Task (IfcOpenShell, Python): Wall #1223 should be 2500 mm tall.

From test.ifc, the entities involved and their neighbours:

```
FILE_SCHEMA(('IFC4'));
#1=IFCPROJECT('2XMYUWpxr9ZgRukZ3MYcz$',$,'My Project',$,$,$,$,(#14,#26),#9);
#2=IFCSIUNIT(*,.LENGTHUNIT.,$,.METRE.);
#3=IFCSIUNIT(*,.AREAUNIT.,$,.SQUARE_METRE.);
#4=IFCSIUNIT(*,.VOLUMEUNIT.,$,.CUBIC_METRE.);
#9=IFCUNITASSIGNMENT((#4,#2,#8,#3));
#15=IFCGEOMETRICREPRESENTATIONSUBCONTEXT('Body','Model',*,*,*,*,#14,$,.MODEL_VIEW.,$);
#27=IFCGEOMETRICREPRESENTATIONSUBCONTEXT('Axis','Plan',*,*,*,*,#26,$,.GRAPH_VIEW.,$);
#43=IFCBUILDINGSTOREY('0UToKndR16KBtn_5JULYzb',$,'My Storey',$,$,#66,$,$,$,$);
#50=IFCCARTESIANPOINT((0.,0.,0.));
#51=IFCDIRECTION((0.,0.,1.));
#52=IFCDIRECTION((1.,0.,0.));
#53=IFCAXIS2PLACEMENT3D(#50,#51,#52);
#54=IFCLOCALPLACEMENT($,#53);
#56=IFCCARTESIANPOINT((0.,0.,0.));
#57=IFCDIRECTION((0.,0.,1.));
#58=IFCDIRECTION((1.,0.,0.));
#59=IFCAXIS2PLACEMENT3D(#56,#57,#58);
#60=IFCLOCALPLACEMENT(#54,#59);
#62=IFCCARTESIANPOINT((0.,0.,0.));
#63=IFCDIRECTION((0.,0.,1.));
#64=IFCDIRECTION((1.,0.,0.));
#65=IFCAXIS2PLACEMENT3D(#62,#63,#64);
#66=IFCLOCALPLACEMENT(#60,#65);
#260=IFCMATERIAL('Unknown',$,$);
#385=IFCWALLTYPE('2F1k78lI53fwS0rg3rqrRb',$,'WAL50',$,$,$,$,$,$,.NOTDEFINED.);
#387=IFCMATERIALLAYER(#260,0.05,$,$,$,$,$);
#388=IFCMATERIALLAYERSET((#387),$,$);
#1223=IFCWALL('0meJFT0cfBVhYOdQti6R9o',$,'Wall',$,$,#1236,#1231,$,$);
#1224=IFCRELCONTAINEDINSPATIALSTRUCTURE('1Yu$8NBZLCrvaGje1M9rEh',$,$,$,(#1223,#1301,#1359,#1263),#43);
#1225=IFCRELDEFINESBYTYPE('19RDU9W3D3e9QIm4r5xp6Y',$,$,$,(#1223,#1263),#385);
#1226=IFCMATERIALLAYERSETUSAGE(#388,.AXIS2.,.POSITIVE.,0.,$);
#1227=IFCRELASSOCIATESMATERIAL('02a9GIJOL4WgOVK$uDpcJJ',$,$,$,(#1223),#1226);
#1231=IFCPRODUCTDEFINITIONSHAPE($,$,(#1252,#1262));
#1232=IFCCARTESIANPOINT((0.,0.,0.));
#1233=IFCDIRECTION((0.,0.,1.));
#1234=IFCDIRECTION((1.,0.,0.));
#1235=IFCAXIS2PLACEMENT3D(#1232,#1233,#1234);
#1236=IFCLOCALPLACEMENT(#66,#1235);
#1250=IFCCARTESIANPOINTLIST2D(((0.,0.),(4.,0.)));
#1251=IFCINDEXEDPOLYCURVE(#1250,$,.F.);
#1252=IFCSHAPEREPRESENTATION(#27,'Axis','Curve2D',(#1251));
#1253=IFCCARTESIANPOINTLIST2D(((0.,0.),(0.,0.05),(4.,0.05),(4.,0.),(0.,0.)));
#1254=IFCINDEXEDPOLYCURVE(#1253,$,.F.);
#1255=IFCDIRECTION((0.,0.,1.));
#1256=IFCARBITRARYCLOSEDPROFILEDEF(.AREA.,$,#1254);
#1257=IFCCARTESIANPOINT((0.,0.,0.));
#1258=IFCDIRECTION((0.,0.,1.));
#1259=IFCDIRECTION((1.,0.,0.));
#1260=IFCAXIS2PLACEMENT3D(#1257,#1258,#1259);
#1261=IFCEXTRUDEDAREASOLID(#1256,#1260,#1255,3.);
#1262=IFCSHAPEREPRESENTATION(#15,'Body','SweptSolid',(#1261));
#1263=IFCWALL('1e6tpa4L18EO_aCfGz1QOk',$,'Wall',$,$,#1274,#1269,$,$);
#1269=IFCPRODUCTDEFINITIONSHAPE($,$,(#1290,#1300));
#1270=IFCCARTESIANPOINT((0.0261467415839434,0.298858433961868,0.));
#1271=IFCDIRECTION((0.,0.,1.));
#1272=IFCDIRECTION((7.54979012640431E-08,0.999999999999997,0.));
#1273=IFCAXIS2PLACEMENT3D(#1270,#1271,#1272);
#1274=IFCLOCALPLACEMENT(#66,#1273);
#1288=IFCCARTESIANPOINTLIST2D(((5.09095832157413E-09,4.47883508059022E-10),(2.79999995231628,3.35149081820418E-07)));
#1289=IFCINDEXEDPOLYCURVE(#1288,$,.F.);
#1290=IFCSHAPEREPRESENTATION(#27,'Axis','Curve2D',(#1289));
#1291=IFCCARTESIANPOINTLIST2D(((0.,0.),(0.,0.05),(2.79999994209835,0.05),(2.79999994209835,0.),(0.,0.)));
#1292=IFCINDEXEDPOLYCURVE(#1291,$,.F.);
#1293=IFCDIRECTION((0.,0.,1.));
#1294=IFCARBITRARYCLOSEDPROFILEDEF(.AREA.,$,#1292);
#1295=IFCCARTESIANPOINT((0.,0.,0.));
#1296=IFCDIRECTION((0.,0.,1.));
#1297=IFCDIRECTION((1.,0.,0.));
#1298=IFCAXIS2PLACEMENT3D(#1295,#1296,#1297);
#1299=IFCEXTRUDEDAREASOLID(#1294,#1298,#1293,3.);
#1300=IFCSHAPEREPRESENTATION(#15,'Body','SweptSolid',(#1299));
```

```python
import ifcopenshell
import ifcopenshell.geom
import ifcopenshell.util.representation
import ifcopenshell.util.shape

model = ifcopenshell.open("test.ifc")
settings = ifcopenshell.geom.settings()


def volume(element):
    """Net volume in cubic metres, openings subtracted."""
    shape = ifcopenshell.geom.create_shape(settings, element)
    return ifcopenshell.util.shape.get_volume(shape.geometry)


wall = model.by_guid("0meJFT0cfBVhYOdQti6R9o")
before = volume(wall)

body = ifcopenshell.util.representation.get_representation(wall, "Model", "Body")
solid = body.Items[0]
old_height = solid.Depth
solid.Depth = 2.5
after = volume(wall)

print(f"height {old_height:g} -> {solid.Depth:g}, volume {before:.3f} -> {after:.3f} m3")

model.write("test-out.ifc")
```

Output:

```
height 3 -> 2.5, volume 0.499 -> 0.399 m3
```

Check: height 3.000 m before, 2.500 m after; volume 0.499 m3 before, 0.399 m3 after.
